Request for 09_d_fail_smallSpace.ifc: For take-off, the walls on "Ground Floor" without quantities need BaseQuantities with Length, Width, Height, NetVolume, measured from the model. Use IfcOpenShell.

First a look at what the model holds.

```python
import ifcopenshell
import ifcopenshell.util.element
import ifcopenshell.util.unit

model = ifcopenshell.open("09_d_fail_smallSpace.ifc")
print(model.schema)
for unit_type in ("LENGTHUNIT", "AREAUNIT", "VOLUMEUNIT"):
    print(unit_type, ifcopenshell.util.unit.calculate_unit_scale(model, unit_type))
storey = next(s for s in model.by_type("IfcBuildingStorey") if s.Name == "Ground Floor")
walls = [e for e in ifcopenshell.util.element.get_decomposition(storey) if e.is_a("IfcWall")]
for e in sorted(walls, key=lambda e: e.id()):
    print(e.id(), e.is_a(), e.Name, list(ifcopenshell.util.element.get_psets(e, qtos_only=True)), sep=" | ")
```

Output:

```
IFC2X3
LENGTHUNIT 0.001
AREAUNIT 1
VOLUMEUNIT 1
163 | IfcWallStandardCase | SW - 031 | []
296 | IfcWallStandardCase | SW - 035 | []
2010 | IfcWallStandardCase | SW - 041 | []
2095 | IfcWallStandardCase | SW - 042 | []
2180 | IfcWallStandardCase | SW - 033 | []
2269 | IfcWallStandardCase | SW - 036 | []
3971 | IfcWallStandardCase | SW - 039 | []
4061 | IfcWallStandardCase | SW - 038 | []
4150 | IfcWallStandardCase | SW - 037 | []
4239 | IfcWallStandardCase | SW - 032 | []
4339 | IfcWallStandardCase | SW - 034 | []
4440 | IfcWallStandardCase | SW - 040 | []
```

```python
import ifcopenshell
import ifcopenshell.api.pset
import ifcopenshell.geom
import ifcopenshell.util.element
import ifcopenshell.util.shape
import ifcopenshell.util.unit

model = ifcopenshell.open("09_d_fail_smallSpace.ifc")
unit_scale = ifcopenshell.util.unit.calculate_unit_scale(model)
volume_scale = ifcopenshell.util.unit.calculate_unit_scale(model, "VOLUMEUNIT")
settings = ifcopenshell.geom.settings()

storey = next(s for s in model.by_type("IfcBuildingStorey") if s.Name == "Ground Floor")
walls = [e for e in ifcopenshell.util.element.get_decomposition(storey) if e.is_a("IfcWall")]

for e in sorted(walls, key=lambda e: e.id()):
    if ifcopenshell.util.element.get_psets(e, qtos_only=True, should_inherit=False):
        continue
    # Geometry comes back in metres, in the element's own axes.
    shape = ifcopenshell.geom.create_shape(settings, e)
    values = {
        "Length": ifcopenshell.util.shape.get_x(shape.geometry) / unit_scale,
        "Width": ifcopenshell.util.shape.get_y(shape.geometry) / unit_scale,
        "Height": ifcopenshell.util.shape.get_z(shape.geometry) / unit_scale,
        "NetVolume": ifcopenshell.util.shape.get_volume(shape.geometry) / volume_scale,
    }
    qto = ifcopenshell.api.pset.add_qto(model, product=e, name="BaseQuantities")
    ifcopenshell.api.pset.edit_qto(model, qto=qto, properties=values)
    print(e.id(), {k: round(v, 3) for k, v in values.items()})

model.write("09_d_fail_smallSpace_updated.ifc")
```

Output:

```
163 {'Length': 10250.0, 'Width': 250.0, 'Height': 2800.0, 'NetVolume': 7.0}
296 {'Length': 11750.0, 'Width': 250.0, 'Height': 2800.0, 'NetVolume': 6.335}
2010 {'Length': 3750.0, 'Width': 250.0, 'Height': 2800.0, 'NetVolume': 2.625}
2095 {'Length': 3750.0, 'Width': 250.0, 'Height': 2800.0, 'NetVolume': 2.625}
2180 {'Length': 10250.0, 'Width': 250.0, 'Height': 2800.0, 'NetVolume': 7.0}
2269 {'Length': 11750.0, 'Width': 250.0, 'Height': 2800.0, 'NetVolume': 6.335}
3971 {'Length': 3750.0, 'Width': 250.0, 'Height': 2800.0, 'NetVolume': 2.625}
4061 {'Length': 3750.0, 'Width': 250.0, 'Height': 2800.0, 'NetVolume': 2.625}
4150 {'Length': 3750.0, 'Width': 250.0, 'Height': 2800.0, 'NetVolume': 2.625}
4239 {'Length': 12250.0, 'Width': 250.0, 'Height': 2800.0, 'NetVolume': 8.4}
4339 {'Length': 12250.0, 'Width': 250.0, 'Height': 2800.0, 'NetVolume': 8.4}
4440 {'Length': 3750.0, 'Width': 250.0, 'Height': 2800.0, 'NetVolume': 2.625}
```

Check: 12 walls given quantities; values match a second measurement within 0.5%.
